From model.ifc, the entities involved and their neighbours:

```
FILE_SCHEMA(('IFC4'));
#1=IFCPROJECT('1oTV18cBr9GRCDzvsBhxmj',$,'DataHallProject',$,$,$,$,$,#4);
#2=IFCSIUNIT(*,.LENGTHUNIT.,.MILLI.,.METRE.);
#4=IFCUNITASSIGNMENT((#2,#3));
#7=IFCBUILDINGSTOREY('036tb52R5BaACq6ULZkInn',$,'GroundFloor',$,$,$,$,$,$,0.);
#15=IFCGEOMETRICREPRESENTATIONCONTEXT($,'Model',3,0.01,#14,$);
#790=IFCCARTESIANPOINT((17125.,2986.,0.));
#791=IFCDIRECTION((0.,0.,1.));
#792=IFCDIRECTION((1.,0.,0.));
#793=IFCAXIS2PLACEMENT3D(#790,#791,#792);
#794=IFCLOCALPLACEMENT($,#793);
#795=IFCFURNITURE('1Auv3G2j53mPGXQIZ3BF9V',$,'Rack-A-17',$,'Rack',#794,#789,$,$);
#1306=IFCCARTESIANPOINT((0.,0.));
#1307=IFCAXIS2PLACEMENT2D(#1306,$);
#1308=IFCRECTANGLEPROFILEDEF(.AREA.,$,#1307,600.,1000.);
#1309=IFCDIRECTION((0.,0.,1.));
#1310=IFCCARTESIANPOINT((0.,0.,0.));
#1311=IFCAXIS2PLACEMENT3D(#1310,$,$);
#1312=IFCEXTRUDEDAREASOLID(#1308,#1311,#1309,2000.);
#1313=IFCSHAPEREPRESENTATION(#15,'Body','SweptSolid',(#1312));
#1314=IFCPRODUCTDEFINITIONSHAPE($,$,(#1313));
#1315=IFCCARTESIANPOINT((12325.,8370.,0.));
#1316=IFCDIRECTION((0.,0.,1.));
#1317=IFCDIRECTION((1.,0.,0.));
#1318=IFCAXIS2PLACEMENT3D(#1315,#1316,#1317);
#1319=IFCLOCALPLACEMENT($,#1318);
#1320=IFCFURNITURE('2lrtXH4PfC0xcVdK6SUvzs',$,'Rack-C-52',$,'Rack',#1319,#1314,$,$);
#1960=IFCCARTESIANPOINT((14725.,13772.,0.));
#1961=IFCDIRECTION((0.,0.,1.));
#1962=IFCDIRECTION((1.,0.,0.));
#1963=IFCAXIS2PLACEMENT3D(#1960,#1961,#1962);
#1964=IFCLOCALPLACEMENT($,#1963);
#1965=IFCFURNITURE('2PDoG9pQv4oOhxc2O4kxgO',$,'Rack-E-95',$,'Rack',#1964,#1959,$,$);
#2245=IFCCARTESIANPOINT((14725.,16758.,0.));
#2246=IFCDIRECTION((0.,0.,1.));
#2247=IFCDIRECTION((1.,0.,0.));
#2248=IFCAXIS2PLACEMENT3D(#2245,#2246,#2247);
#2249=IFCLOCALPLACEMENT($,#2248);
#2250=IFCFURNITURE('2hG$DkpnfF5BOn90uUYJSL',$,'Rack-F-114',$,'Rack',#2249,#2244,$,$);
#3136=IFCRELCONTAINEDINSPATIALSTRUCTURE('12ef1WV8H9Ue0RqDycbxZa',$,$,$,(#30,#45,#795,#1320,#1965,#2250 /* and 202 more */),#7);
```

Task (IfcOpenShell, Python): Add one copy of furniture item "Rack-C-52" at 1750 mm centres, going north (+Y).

```python
import numpy as np
import ifcopenshell
import ifcopenshell.api.geometry
import ifcopenshell.api.root
import ifcopenshell.util.element
import ifcopenshell.util.placement
import ifcopenshell.util.unit

model = ifcopenshell.open("model.ifc")
unit_scale = ifcopenshell.util.unit.calculate_unit_scale(model)

source = model.by_guid("2lrtXH4PfC0xcVdK6SUvzs")
base = ifcopenshell.util.placement.get_local_placement(source.ObjectPlacement)
step = np.array([0.0, 1.0, 0.0]) * 1.75 / unit_scale

for i in range(1, 2):
    copy = ifcopenshell.api.root.copy_class(model, product=source)
    copy.Representation = ifcopenshell.util.element.copy_deep(
        model, source.Representation, exclude=["IfcGeometricRepresentationContext", "IfcRepresentationMap"]
    )
    matrix = base.copy()
    matrix[:3, 3] += i * step
    print("added at", matrix[:3, 3].round(3) + 0.0)
    ifcopenshell.api.geometry.edit_object_placement(model, product=copy, matrix=matrix, is_si=False)

model.write("model_rev.ifc")
```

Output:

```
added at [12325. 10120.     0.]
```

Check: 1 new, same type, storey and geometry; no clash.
